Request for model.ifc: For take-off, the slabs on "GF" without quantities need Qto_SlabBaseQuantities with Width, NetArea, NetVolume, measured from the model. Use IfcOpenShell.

First a look at what the model holds.

```python
import ifcopenshell
import ifcopenshell.util.element
import ifcopenshell.util.unit

model = ifcopenshell.open("model.ifc")
print(model.schema)
for unit_type in ("LENGTHUNIT", "AREAUNIT", "VOLUMEUNIT"):
    print(unit_type, ifcopenshell.util.unit.calculate_unit_scale(model, unit_type))
storey = next(s for s in model.by_type("IfcBuildingStorey") if s.Name == "GF")
slabs = [e for e in ifcopenshell.util.element.get_decomposition(storey) if e.is_a("IfcSlab")]
for e in sorted(slabs, key=lambda e: e.id()):
    print(e.id(), e.is_a(), e.Name, list(ifcopenshell.util.element.get_psets(e, qtos_only=True)), sep=" | ")
```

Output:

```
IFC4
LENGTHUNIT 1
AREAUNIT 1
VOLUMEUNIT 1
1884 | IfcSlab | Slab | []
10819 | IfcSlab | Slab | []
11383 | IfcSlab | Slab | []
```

```python
import ifcopenshell
import ifcopenshell.api.pset
import ifcopenshell.geom
import ifcopenshell.util.element
import ifcopenshell.util.shape
import ifcopenshell.util.unit

model = ifcopenshell.open("model.ifc")
unit_scale = ifcopenshell.util.unit.calculate_unit_scale(model)
area_scale = ifcopenshell.util.unit.calculate_unit_scale(model, "AREAUNIT")
volume_scale = ifcopenshell.util.unit.calculate_unit_scale(model, "VOLUMEUNIT")
settings = ifcopenshell.geom.settings()

storey = next(s for s in model.by_type("IfcBuildingStorey") if s.Name == "GF")
slabs = [e for e in ifcopenshell.util.element.get_decomposition(storey) if e.is_a("IfcSlab")]

for e in sorted(slabs, key=lambda e: e.id()):
    if ifcopenshell.util.element.get_psets(e, qtos_only=True, should_inherit=False):
        continue
    # Geometry comes back in metres, in the element's own axes.
    shape = ifcopenshell.geom.create_shape(settings, e)
    values = {
        "Width": ifcopenshell.util.shape.get_z(shape.geometry) / unit_scale,
        "NetArea": ifcopenshell.util.shape.get_footprint_area(shape.geometry) / area_scale,
        "NetVolume": ifcopenshell.util.shape.get_volume(shape.geometry) / volume_scale,
    }
    qto = ifcopenshell.api.pset.add_qto(model, product=e, name="Qto_SlabBaseQuantities")
    ifcopenshell.api.pset.edit_qto(model, qto=qto, properties=values)
    print(e.id(), {k: round(v, 3) for k, v in values.items()})

model.write("model-out.ifc")
```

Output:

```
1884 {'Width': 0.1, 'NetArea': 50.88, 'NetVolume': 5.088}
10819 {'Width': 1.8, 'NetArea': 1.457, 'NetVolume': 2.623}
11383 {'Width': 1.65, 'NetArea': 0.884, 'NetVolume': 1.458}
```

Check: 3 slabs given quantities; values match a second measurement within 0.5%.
